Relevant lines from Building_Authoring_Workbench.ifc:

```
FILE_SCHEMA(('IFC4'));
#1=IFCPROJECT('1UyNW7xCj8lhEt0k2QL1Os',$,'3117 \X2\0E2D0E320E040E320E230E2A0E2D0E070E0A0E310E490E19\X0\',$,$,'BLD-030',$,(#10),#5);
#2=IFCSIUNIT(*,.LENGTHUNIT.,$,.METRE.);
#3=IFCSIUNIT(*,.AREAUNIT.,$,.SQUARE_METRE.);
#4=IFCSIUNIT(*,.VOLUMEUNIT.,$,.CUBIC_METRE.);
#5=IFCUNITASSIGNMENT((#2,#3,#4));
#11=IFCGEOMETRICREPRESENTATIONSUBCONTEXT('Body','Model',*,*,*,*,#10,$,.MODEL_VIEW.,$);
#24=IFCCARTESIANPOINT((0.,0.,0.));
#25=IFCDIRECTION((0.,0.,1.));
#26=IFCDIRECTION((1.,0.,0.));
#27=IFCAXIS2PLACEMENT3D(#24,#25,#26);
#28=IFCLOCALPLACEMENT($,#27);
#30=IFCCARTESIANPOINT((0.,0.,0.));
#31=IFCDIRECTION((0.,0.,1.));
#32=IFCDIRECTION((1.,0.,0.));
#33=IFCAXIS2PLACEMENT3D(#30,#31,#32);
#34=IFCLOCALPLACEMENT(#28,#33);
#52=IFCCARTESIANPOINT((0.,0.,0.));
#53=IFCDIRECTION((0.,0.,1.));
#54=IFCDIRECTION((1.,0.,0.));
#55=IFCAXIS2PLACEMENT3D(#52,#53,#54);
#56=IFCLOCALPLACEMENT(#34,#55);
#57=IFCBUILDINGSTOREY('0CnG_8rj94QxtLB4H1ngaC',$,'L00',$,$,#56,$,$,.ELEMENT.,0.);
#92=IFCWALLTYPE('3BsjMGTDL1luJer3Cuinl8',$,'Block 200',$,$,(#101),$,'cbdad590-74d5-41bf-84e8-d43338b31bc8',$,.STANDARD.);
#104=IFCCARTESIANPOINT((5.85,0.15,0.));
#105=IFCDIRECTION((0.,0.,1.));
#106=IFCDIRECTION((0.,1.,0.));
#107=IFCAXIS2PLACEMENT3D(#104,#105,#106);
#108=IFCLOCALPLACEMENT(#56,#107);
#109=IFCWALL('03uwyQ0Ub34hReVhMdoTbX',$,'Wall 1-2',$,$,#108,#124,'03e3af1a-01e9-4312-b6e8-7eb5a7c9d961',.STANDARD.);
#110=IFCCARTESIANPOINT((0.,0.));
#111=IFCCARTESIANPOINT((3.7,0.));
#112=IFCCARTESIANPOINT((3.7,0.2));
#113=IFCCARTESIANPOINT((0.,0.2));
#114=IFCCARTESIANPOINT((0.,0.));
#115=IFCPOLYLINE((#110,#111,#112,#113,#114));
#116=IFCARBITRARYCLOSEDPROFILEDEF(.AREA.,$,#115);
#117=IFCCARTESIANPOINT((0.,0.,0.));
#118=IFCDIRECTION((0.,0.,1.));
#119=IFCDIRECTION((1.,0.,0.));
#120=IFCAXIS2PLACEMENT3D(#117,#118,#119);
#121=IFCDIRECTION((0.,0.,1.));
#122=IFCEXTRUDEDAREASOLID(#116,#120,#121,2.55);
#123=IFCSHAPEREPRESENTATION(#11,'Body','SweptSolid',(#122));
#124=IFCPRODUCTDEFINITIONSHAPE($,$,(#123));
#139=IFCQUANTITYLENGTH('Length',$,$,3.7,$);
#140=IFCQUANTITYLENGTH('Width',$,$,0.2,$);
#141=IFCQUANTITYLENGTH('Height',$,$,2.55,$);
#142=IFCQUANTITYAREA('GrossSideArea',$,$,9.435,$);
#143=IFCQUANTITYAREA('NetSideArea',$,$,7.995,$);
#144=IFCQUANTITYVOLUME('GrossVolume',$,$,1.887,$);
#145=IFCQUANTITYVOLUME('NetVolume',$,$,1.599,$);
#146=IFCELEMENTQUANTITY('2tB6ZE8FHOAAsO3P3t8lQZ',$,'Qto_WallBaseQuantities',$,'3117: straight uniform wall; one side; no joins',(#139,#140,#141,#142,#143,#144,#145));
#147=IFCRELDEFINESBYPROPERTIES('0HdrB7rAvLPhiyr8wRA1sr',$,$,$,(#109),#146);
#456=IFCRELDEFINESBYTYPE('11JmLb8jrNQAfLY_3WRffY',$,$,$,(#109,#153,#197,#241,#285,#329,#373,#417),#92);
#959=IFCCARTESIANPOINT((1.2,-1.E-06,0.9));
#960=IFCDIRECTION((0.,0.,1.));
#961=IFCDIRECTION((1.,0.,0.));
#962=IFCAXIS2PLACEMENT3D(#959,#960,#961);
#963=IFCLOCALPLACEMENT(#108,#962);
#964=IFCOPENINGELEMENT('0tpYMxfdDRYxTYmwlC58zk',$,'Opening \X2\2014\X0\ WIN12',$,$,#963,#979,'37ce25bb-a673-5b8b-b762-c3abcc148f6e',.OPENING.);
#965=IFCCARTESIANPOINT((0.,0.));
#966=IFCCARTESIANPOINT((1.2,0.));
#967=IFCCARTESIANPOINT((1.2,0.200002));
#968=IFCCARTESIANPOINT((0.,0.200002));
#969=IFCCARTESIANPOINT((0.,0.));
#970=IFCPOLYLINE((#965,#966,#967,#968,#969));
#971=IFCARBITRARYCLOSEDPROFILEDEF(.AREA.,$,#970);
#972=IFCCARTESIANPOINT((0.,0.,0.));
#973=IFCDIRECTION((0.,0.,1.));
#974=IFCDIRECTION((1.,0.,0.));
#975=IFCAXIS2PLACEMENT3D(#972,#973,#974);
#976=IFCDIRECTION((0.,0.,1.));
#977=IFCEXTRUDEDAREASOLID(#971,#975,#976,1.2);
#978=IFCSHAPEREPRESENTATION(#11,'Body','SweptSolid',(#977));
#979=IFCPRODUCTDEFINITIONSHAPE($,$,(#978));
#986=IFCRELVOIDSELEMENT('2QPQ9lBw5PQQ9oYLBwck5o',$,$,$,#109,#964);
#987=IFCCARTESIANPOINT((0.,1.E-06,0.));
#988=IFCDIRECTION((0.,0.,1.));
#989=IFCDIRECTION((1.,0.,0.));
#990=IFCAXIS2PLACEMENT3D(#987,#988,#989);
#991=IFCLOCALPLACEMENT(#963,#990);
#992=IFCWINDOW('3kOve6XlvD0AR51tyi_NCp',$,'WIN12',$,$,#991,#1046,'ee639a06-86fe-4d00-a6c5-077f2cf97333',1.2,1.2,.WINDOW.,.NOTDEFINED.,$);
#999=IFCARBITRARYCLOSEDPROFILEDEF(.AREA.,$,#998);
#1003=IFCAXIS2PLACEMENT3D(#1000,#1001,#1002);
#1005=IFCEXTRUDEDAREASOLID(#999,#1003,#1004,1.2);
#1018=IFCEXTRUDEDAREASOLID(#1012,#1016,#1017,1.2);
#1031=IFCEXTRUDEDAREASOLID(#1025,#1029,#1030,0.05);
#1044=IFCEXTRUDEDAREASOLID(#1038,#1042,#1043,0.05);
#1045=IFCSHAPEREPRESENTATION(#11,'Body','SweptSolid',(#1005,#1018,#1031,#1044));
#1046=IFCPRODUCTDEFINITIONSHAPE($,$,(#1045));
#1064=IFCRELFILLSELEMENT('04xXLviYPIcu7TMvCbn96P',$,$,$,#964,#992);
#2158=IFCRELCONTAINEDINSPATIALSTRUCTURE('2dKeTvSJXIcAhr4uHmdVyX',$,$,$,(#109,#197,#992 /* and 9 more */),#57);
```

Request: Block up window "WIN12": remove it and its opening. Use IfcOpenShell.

```python
import ifcopenshell
import ifcopenshell.api.feature
import ifcopenshell.api.pset
import ifcopenshell.api.root
import ifcopenshell.geom
import ifcopenshell.util.element
import ifcopenshell.util.shape
import ifcopenshell.util.unit

model = ifcopenshell.open("Building_Authoring_Workbench.ifc")
area_scale = ifcopenshell.util.unit.calculate_unit_scale(model, "AREAUNIT")
volume_scale = ifcopenshell.util.unit.calculate_unit_scale(model, "VOLUMEUNIT")
settings = ifcopenshell.geom.settings()


def volume(element):
    """Net volume in cubic metres, openings subtracted."""
    shape = ifcopenshell.geom.create_shape(settings, element)
    return ifcopenshell.util.shape.get_volume(shape.geometry)


window = model.by_id(992)
opening = window.FillsVoids[0].RelatingOpeningElement
wall = opening.VoidsElements[0].RelatingBuildingElement
before = volume(wall)

ifcopenshell.api.root.remove_product(model, product=window)
ifcopenshell.api.feature.remove_feature(model, feature=opening)

after = volume(wall)
thickness = 0.2  # wall thickness in metres

# Update the wall's stored quantities.
qto = model.by_id(ifcopenshell.util.element.get_pset(wall, "Qto_WallBaseQuantities", should_inherit=False)["id"])
ifcopenshell.api.pset.edit_qto(model, qto=qto, properties={
    "NetSideArea": after / thickness / area_scale,
    "NetVolume": after / volume_scale,
})

print(f"wall volume {before:.3f} -> {after:.3f} m3")

model.write("Building_Authoring_Workbench_v2.ifc")
```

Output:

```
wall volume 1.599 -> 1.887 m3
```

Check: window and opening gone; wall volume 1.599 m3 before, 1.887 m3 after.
